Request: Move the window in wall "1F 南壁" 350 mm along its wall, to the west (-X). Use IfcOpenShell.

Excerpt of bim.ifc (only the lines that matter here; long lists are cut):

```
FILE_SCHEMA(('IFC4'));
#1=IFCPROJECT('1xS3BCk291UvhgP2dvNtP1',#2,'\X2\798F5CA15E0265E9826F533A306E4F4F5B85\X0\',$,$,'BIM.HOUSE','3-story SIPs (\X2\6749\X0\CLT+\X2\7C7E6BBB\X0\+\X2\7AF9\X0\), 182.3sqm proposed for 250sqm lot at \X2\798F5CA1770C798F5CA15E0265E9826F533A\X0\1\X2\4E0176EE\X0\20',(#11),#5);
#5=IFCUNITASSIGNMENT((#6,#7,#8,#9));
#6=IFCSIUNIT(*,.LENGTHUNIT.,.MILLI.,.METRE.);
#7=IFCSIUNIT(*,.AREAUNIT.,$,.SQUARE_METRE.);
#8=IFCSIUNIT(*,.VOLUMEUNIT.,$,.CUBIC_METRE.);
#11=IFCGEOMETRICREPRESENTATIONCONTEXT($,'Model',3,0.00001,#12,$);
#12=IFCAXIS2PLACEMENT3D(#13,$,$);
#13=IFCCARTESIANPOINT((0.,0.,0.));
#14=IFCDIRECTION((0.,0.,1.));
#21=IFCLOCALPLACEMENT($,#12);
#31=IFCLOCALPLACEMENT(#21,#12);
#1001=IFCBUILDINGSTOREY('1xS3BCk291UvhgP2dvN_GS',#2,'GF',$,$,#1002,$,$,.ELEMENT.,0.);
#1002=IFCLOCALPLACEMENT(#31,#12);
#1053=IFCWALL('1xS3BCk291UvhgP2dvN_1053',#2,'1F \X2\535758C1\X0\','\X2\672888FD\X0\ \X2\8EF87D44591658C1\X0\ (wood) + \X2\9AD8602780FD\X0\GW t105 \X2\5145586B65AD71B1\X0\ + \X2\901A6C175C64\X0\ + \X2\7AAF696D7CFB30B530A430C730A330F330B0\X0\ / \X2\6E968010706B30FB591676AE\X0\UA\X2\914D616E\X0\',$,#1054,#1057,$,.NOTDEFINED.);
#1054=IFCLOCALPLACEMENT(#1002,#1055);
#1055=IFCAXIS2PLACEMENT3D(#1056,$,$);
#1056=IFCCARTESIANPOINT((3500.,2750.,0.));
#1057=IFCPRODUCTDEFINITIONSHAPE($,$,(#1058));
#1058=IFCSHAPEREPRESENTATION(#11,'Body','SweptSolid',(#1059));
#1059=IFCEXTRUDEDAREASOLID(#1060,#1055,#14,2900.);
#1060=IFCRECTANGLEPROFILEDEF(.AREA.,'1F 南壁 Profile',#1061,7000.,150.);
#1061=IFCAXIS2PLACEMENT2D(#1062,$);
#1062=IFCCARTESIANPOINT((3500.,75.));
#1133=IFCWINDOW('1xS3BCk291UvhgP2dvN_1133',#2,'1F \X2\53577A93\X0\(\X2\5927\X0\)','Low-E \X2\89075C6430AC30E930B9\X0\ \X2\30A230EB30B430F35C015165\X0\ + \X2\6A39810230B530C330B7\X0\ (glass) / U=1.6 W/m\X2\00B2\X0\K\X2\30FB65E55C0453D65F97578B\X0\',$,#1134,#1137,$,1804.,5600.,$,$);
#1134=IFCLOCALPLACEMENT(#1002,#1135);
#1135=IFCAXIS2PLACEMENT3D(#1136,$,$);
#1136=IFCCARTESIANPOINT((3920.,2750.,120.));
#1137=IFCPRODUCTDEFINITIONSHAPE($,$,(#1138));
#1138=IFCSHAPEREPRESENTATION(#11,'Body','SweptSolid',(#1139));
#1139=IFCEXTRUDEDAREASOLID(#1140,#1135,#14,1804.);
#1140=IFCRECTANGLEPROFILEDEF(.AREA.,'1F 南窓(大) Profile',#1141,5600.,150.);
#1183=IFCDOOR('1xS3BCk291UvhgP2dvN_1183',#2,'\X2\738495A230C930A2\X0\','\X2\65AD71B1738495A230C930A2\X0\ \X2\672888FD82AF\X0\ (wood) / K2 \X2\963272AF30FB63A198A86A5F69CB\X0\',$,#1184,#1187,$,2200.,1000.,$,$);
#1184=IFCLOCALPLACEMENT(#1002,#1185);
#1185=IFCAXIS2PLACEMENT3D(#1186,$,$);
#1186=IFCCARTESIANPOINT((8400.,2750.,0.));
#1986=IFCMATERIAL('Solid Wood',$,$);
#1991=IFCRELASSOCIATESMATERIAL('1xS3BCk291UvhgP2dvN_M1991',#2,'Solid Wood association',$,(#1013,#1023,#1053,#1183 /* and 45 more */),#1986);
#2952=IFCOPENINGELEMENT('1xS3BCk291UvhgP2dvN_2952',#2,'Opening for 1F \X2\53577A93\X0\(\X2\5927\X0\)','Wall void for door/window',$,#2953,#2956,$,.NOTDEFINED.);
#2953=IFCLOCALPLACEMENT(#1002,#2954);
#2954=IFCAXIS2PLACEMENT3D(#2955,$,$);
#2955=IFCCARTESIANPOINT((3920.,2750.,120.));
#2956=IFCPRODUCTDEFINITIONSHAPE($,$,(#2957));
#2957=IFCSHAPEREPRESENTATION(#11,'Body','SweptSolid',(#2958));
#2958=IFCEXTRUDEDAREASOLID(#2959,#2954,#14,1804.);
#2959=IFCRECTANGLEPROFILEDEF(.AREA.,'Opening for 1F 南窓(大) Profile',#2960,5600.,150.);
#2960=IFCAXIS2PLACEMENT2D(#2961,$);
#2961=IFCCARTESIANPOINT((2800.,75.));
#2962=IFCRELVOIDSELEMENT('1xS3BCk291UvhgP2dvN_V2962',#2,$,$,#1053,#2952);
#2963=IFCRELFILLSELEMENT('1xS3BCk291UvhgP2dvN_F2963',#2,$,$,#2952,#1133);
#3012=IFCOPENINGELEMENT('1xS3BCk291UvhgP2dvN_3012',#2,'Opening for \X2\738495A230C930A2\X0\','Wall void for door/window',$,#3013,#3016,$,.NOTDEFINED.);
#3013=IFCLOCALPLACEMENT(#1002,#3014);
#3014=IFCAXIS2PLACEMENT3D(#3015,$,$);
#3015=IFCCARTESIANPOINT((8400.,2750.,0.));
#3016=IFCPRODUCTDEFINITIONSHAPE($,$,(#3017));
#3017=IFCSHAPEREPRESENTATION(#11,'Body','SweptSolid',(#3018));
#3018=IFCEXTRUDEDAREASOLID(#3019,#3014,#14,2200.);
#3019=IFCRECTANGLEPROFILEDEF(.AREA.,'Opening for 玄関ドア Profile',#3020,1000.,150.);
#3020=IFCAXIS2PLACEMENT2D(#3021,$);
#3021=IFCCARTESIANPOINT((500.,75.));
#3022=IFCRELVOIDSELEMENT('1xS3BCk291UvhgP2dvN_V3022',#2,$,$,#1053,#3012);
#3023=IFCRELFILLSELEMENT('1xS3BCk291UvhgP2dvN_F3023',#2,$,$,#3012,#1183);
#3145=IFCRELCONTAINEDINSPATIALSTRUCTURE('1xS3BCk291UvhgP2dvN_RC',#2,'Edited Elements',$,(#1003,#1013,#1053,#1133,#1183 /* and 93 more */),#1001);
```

```python
import ifcopenshell
import ifcopenshell.api.geometry
import ifcopenshell.util.placement
import ifcopenshell.util.unit

model = ifcopenshell.open("bim.ifc")
unit_scale = ifcopenshell.util.unit.calculate_unit_scale(model)

window = model.by_guid("1xS3BCk291UvhgP2dvN_1133")
opening = window.FillsVoids[0].RelatingOpeningElement
wall = opening.VoidsElements[0].RelatingBuildingElement

wall_matrix = ifcopenshell.util.placement.get_local_placement(wall.ObjectPlacement)
shift = wall_matrix[:3, 0] * -0.35 / unit_scale
before = ifcopenshell.util.placement.get_local_placement(window.ObjectPlacement)[:3, 3].copy()

# The window is not placed relative to its opening, so move both.
for product in (opening, window):
    matrix = ifcopenshell.util.placement.get_local_placement(product.ObjectPlacement)
    matrix[:3, 3] += shift
    ifcopenshell.api.geometry.edit_object_placement(model, product=product, matrix=matrix, is_si=False)

after = ifcopenshell.util.placement.get_local_placement(window.ObjectPlacement)[:3, 3]
print("window moved by", (after - before).round(3) + 0.0)

model.write("bim-out.ifc")
```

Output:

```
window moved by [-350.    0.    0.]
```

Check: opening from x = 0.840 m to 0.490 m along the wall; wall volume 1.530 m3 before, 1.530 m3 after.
